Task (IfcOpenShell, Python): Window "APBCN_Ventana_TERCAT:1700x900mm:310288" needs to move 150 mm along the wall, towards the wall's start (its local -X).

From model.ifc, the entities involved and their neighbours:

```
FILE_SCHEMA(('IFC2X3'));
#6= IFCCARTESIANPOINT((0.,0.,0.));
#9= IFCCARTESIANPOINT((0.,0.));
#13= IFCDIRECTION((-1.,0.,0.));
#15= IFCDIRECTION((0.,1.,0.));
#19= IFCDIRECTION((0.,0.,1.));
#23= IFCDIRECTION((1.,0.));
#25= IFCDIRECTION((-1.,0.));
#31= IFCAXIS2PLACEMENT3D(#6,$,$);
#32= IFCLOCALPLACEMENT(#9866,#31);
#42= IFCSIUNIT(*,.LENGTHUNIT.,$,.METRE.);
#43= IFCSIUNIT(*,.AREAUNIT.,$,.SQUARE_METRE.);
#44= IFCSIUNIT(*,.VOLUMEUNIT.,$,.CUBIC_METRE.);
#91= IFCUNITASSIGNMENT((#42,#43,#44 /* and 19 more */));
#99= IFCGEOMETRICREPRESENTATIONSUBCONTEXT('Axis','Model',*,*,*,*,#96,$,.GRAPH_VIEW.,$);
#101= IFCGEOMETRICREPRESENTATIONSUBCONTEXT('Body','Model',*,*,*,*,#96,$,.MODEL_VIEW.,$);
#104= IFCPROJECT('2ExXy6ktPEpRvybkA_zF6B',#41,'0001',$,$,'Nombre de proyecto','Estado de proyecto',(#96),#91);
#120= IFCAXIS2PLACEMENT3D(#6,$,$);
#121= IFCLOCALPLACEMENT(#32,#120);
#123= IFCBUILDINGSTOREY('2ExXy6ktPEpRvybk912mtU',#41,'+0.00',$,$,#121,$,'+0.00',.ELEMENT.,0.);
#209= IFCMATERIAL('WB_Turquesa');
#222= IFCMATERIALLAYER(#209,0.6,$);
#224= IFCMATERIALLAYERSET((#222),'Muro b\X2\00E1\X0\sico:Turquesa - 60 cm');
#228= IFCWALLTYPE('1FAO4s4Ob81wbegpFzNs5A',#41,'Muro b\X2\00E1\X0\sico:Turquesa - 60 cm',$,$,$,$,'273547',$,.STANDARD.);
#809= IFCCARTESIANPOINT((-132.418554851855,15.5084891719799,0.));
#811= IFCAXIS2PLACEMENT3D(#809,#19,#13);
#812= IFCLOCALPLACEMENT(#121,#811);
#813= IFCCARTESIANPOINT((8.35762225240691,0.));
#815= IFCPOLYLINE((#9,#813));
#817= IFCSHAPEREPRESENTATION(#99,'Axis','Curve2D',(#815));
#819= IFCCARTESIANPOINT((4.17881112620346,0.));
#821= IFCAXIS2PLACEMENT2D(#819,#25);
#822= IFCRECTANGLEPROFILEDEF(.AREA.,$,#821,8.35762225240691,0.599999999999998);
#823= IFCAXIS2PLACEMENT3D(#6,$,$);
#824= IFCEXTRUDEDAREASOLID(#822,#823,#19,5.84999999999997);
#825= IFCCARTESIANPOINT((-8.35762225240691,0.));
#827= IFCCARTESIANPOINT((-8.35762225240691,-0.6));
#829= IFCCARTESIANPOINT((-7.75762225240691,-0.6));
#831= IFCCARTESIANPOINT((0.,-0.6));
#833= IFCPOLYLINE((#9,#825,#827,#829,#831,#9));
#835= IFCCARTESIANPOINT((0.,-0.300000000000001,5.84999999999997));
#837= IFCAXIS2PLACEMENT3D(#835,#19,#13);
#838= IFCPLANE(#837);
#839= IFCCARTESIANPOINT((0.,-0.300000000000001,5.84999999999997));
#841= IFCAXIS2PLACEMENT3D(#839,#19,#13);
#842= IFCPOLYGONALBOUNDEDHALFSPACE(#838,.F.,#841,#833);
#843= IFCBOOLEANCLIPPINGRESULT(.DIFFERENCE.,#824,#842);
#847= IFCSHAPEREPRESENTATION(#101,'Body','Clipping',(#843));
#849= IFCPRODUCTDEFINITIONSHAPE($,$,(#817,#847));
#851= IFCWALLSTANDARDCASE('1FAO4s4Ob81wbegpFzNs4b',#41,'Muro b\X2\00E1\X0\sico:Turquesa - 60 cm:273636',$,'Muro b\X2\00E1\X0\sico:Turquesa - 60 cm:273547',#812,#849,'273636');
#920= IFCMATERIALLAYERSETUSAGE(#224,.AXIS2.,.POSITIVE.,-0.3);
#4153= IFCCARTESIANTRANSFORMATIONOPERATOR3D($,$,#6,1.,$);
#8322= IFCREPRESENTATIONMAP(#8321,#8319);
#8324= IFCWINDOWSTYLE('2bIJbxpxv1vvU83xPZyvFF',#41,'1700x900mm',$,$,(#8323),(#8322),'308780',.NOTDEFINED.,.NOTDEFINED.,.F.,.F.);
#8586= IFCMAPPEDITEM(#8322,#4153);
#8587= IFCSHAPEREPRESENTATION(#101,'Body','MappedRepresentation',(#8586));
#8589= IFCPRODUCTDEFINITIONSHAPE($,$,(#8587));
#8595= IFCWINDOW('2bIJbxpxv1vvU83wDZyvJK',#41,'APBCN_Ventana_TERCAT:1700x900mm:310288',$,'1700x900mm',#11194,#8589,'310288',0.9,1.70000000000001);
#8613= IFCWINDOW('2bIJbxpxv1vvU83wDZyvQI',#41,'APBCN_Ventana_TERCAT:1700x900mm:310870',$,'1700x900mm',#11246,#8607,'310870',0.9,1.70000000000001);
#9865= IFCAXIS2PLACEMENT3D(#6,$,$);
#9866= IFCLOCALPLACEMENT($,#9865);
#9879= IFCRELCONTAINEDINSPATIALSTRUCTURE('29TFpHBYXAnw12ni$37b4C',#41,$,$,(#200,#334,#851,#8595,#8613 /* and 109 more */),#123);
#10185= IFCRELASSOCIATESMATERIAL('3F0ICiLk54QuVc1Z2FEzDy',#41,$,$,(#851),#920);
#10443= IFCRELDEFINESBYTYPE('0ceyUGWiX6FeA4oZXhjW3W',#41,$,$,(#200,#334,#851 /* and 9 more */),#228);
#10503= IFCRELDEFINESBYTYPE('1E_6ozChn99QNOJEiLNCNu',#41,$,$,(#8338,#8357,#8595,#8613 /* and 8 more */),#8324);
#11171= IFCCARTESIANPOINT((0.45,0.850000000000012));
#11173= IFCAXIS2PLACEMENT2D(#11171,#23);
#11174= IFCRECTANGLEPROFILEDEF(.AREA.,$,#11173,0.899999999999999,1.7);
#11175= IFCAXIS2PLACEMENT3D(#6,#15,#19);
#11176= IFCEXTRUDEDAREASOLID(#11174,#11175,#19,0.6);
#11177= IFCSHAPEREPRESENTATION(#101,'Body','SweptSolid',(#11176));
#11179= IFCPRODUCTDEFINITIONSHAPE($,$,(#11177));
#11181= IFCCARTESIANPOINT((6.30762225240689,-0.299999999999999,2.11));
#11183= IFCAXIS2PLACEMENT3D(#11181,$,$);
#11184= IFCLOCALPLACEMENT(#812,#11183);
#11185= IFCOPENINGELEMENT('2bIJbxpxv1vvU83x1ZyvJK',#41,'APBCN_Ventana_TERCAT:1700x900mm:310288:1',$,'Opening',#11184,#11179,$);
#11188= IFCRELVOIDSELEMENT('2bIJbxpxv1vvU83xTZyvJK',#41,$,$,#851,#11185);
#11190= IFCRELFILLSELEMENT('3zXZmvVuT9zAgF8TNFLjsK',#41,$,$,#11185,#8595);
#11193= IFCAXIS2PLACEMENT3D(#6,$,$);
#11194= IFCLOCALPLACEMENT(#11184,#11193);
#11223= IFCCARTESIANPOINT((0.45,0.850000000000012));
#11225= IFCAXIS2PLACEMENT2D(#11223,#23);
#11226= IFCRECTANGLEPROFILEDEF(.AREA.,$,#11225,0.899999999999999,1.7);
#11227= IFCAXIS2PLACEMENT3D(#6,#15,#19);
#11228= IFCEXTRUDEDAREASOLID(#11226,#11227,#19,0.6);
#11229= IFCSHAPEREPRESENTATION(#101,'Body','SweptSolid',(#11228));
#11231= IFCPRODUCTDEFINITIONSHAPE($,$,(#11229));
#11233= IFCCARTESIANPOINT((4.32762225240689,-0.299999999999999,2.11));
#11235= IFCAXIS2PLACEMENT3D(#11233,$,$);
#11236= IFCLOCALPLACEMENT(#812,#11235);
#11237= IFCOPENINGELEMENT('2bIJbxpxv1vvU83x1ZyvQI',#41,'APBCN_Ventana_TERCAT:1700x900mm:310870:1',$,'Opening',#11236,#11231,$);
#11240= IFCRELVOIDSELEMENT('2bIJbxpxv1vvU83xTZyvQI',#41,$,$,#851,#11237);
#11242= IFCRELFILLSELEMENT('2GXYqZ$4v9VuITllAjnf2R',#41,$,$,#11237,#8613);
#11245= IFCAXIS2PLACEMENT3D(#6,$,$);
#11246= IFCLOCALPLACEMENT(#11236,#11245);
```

```python
import ifcopenshell
import ifcopenshell.api.geometry
import ifcopenshell.util.placement
import ifcopenshell.util.unit

model = ifcopenshell.open("model.ifc")
unit_scale = ifcopenshell.util.unit.calculate_unit_scale(model)

window = model.by_guid("2bIJbxpxv1vvU83wDZyvJK")
opening = window.FillsVoids[0].RelatingOpeningElement
wall = opening.VoidsElements[0].RelatingBuildingElement

wall_matrix = ifcopenshell.util.placement.get_local_placement(wall.ObjectPlacement)
shift = wall_matrix[:3, 0] * -0.15 / unit_scale
before = ifcopenshell.util.placement.get_local_placement(window.ObjectPlacement)[:3, 3].copy()

# The window is placed relative to its opening, so it follows when the opening moves.
matrix = ifcopenshell.util.placement.get_local_placement(opening.ObjectPlacement)
matrix[:3, 3] += shift
ifcopenshell.api.geometry.edit_object_placement(
    model, product=opening, matrix=matrix, is_si=False, should_transform_children=True
)

after = ifcopenshell.util.placement.get_local_placement(window.ObjectPlacement)[:3, 3]
print("window moved by", (after - before).round(3) + 0.0)

model.write("model_updated.ifc")
```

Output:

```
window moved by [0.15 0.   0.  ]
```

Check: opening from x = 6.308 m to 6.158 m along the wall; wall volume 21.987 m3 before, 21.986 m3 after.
